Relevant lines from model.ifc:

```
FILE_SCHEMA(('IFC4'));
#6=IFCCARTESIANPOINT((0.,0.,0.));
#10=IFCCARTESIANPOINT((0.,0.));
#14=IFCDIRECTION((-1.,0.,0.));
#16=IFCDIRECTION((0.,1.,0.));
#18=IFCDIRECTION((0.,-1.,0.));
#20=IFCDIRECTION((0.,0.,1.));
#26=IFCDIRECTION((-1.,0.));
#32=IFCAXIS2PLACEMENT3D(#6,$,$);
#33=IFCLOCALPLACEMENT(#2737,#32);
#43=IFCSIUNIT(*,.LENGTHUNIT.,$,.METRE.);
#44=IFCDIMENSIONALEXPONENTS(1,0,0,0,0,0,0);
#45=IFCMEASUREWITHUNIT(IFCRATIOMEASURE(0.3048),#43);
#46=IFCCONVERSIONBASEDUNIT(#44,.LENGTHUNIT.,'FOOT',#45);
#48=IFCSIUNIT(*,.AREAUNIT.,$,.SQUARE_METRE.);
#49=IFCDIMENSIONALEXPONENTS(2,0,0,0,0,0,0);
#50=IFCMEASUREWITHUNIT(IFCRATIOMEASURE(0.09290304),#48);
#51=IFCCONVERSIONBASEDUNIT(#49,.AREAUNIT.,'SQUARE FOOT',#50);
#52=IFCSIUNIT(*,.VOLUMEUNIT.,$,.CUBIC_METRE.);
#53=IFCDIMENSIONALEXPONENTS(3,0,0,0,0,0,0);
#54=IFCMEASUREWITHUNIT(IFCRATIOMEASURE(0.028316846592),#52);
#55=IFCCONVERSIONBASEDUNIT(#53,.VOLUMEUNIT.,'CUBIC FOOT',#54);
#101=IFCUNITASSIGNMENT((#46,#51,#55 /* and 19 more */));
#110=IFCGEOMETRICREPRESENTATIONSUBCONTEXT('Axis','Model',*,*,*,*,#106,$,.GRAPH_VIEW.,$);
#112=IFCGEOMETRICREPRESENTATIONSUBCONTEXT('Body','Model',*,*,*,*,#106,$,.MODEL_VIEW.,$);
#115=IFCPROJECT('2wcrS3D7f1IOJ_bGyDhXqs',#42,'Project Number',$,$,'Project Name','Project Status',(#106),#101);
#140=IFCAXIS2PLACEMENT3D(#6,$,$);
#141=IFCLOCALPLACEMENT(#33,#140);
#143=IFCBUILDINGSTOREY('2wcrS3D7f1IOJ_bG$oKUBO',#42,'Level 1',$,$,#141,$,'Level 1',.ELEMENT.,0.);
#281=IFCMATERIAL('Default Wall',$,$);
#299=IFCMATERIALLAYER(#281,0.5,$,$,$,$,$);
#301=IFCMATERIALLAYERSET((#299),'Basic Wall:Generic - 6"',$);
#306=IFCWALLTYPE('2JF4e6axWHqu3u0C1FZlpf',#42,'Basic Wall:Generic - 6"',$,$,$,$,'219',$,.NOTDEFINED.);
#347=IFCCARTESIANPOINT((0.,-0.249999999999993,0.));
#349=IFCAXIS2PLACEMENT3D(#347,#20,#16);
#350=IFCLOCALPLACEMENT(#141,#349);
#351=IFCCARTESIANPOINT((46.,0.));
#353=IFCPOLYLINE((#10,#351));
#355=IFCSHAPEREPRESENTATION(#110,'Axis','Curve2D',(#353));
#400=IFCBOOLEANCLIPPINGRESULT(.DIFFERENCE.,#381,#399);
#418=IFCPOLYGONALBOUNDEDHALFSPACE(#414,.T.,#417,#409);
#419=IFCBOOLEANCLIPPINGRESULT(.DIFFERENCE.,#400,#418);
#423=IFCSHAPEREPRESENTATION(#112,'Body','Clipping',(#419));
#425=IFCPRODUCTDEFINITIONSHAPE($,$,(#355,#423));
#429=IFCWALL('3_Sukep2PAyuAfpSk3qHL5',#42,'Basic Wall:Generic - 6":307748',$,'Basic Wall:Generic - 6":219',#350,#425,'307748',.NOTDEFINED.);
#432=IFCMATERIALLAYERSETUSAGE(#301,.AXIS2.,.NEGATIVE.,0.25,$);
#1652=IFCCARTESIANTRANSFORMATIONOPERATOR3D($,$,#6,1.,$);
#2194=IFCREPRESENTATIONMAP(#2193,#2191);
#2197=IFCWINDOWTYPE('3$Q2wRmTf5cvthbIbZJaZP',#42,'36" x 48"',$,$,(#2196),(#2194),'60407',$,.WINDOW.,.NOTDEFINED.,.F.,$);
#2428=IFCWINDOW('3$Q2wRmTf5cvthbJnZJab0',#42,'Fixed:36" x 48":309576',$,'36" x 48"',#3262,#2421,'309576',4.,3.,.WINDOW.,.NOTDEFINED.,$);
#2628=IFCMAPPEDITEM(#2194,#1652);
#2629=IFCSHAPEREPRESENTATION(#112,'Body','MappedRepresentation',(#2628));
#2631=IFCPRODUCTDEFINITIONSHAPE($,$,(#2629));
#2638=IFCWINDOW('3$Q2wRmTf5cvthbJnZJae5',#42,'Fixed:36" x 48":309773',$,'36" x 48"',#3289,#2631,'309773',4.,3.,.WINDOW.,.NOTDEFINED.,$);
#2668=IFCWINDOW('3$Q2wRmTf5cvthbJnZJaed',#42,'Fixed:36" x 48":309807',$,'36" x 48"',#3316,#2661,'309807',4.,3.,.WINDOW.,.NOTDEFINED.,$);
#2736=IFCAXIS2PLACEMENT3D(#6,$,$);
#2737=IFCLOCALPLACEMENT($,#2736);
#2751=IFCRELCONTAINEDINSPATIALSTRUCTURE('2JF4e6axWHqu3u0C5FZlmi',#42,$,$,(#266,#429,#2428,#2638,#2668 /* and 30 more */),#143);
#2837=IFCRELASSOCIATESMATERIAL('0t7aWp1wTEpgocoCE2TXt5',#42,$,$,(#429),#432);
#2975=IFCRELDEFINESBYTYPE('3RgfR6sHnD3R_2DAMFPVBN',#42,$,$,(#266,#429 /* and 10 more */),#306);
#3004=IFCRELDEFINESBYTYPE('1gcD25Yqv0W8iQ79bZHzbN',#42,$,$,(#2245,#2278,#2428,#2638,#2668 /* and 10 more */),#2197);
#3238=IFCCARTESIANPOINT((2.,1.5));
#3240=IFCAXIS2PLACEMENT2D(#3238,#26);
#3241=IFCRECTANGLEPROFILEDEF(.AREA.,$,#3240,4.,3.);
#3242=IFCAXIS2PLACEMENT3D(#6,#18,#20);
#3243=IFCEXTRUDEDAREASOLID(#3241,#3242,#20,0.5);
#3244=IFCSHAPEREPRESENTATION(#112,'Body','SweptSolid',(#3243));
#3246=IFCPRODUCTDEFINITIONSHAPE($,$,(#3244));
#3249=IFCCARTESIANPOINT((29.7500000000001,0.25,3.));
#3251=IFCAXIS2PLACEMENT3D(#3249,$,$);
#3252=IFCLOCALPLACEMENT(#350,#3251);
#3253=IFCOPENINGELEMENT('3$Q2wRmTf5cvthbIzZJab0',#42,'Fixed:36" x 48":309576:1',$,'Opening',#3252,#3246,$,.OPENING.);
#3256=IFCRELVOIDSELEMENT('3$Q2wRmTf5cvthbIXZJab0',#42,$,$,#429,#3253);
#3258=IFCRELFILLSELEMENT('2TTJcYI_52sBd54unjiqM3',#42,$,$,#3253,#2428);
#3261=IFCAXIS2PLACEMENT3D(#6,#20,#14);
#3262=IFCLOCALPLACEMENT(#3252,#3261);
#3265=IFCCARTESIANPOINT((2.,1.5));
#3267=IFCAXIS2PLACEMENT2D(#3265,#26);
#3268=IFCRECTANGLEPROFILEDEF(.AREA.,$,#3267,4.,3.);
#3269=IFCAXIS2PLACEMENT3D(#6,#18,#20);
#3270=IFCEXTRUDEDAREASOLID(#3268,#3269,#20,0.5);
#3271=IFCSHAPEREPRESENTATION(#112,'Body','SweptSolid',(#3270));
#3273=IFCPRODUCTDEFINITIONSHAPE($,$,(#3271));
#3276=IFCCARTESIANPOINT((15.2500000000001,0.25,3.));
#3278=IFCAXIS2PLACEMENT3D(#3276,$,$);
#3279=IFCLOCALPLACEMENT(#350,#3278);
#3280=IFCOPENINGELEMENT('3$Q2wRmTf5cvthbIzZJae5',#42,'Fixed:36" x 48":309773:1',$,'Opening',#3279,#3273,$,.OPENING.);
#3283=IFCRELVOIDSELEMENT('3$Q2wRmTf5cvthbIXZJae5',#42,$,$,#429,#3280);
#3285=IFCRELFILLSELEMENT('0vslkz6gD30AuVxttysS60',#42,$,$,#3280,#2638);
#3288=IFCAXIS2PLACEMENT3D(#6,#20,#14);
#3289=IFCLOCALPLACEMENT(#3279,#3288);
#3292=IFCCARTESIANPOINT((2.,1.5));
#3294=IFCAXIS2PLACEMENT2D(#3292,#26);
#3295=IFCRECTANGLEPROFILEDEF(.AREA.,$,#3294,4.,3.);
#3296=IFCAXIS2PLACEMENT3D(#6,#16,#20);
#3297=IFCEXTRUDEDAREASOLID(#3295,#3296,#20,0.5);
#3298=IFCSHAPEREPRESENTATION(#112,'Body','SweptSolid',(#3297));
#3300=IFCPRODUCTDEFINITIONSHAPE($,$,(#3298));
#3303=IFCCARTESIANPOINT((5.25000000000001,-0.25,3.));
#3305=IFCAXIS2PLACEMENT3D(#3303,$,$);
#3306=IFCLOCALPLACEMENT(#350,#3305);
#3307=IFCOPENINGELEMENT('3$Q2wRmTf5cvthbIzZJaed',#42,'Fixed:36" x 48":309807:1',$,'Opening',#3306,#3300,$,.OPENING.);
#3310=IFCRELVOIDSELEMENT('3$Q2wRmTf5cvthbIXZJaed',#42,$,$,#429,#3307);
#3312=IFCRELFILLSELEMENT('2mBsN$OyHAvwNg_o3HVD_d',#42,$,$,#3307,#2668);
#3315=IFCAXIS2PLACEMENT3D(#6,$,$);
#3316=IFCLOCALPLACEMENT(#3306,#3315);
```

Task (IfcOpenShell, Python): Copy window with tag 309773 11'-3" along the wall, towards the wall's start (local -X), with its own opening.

```python
import ifcopenshell
import ifcopenshell.api.feature
import ifcopenshell.api.geometry
import ifcopenshell.api.root
import ifcopenshell.geom
import ifcopenshell.util.element
import ifcopenshell.util.placement
import ifcopenshell.util.shape
import ifcopenshell.util.unit

model = ifcopenshell.open("model.ifc")
unit_scale = ifcopenshell.util.unit.calculate_unit_scale(model)
settings = ifcopenshell.geom.settings()


def volume(element):
    """Net volume in cubic metres, openings subtracted."""
    shape = ifcopenshell.geom.create_shape(settings, element)
    return ifcopenshell.util.shape.get_volume(shape.geometry)


def reuse_history(source, copy):
    """copy_class also copies each property set's owner history, people and application; keep the originals."""
    for rel in copy.IsDefinedBy:
        if rel.is_a("IfcRelDefinesByProperties") and (history := rel.RelatingPropertyDefinition.OwnerHistory):
            rel.RelatingPropertyDefinition.OwnerHistory = source.OwnerHistory
            ifcopenshell.util.element.remove_deep2(model, history)


window = model.by_guid("3$Q2wRmTf5cvthbJnZJae5")
opening = window.FillsVoids[0].RelatingOpeningElement
wall = opening.VoidsElements[0].RelatingBuildingElement
before = volume(wall)
shift = ifcopenshell.util.placement.get_local_placement(wall.ObjectPlacement)[:3, 0] * -135 * 0.0254 / unit_scale

# copy_class copies the void relationship, type, container and properties, but no geometry.
new_opening = ifcopenshell.api.root.copy_class(model, product=opening)
new_opening.Representation = ifcopenshell.util.element.copy_deep(
    model, opening.Representation, exclude=["IfcGeometricRepresentationContext", "IfcRepresentationMap"]
)
new_opening.Name = 'Fixed:36" x 48"'
new_window = ifcopenshell.api.root.copy_class(model, product=window)
new_window.Representation = ifcopenshell.util.element.copy_deep(
    model, window.Representation, exclude=["IfcGeometricRepresentationContext", "IfcRepresentationMap"]
)
new_window.Name = 'Fixed:36" x 48"'
new_window.Tag = None
reuse_history(window, new_window)
ifcopenshell.api.feature.add_filling(model, opening=new_opening, element=new_window)

for old, new in ((opening, new_opening), (window, new_window)):
    matrix = ifcopenshell.util.placement.get_local_placement(old.ObjectPlacement)
    matrix[:3, 3] += shift
    ifcopenshell.api.geometry.edit_object_placement(model, product=new, matrix=matrix, is_si=False)

after = volume(wall)

print(f"wall volume {before:.3f} -> {after:.3f} m3")

model.write("model_v2.ifc")
```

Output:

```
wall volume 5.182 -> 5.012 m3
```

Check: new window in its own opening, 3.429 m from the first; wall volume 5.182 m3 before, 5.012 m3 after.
